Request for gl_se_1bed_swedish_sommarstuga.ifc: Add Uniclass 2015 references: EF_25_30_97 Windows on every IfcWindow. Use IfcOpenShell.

First a look at what the model holds.

```python
import ifcopenshell

model = ifcopenshell.open("gl_se_1bed_swedish_sommarstuga.ifc")
print(model.schema)
print("classifications:", [c.Name for c in model.by_type("IfcClassification")])
for ifc_class in ("IfcDoor", "IfcRoof", "IfcStair", "IfcWall", "IfcWindow"):
    print(ifc_class, len(model.by_type(ifc_class)))
```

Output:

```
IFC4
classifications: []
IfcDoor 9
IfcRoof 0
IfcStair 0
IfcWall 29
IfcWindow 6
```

```python
import ifcopenshell
import ifcopenshell.api.classification

model = ifcopenshell.open("gl_se_1bed_swedish_sommarstuga.ifc")

system = ifcopenshell.api.classification.add_classification(model, classification="Uniclass 2015")

codes = {
    "IfcWindow": ("EF_25_30_97", "Windows"),
}
for ifc_class, (code, name) in codes.items():
    products = model.by_type(ifc_class)
    ifcopenshell.api.classification.add_reference(
        model, products=products, classification=system, identification=code, name=name
    )
    print(code, len(products))

model.write("gl_se_1bed_swedish_sommarstuga_edited.ifc")
```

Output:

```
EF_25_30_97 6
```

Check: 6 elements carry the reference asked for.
